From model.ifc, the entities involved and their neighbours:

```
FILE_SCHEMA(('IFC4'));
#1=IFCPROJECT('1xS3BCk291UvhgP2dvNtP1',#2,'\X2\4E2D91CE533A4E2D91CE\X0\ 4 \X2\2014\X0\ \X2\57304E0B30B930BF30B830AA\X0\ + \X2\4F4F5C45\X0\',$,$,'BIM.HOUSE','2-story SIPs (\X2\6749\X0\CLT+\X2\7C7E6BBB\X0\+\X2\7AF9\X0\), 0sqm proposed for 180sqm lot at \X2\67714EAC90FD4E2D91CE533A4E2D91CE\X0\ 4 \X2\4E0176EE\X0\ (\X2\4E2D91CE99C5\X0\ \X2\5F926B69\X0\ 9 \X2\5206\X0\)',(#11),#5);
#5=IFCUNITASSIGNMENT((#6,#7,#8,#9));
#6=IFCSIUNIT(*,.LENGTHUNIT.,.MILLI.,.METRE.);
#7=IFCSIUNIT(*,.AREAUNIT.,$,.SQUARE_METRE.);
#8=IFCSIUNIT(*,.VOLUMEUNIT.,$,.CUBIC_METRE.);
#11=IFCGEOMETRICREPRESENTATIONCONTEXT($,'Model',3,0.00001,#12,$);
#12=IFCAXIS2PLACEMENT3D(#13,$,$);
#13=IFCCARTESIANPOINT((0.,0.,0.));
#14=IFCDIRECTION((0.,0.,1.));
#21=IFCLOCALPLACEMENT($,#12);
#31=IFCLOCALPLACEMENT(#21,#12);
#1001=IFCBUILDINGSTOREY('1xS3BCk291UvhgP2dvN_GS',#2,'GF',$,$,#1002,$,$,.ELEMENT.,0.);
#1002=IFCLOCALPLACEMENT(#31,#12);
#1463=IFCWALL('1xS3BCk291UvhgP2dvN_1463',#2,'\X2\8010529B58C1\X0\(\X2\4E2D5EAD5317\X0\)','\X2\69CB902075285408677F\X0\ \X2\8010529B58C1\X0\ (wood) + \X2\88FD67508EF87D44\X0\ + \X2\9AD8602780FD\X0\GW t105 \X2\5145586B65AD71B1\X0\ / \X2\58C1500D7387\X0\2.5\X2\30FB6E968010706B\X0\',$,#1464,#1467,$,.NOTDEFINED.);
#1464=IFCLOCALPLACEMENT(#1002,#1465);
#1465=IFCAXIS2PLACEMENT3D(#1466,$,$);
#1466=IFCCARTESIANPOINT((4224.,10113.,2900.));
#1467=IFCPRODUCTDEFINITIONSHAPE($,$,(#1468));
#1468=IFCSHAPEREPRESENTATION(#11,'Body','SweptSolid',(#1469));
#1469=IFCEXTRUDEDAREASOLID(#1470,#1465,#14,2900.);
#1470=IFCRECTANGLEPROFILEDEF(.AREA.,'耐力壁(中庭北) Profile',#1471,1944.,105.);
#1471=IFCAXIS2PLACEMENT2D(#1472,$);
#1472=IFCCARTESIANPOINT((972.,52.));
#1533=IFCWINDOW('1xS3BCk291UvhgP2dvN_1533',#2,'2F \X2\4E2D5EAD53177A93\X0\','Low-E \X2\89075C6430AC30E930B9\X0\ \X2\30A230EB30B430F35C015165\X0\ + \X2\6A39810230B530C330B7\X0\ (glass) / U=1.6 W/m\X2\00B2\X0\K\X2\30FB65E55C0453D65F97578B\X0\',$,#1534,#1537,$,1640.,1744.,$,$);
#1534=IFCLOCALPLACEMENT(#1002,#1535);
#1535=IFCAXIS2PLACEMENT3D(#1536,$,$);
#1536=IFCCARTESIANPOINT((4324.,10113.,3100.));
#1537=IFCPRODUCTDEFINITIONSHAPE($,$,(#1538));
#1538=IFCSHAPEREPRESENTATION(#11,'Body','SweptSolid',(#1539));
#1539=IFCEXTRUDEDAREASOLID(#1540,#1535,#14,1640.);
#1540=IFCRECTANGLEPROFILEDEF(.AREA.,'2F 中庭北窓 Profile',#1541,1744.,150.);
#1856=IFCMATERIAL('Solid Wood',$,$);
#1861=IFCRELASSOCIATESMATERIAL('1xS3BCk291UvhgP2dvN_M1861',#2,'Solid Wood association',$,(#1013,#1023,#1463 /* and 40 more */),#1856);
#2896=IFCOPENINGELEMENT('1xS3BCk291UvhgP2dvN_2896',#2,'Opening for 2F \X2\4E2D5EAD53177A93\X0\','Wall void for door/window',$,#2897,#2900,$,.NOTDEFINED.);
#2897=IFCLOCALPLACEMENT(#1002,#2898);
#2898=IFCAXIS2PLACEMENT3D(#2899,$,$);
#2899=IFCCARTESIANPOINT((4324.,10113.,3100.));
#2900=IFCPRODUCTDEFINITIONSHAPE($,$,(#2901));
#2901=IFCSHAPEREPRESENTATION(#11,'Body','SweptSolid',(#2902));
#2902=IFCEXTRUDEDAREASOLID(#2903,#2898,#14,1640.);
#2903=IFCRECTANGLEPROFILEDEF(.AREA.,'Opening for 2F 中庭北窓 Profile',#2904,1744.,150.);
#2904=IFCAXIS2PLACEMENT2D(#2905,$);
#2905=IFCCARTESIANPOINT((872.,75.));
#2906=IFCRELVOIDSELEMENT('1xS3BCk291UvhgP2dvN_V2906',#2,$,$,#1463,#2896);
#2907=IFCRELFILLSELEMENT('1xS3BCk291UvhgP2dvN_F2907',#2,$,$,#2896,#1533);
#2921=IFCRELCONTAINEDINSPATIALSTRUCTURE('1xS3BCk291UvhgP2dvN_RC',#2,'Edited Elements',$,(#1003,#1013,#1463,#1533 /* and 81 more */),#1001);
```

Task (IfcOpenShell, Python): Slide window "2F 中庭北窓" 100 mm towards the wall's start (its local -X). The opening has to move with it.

```python
import ifcopenshell
import ifcopenshell.api.geometry
import ifcopenshell.util.placement

model = ifcopenshell.open("model.ifc")

window = model.by_id(1533)
opening = window.FillsVoids[0].RelatingOpeningElement
wall = opening.VoidsElements[0].RelatingBuildingElement

wall_matrix = ifcopenshell.util.placement.get_local_placement(wall.ObjectPlacement)
shift = wall_matrix[:3, 0] * -100.0
before = ifcopenshell.util.placement.get_local_placement(window.ObjectPlacement)[:3, 3].copy()

# The window is not placed relative to its opening, so move both.
for product in (opening, window):
    matrix = ifcopenshell.util.placement.get_local_placement(product.ObjectPlacement)
    matrix[:3, 3] += shift
    ifcopenshell.api.geometry.edit_object_placement(model, product=product, matrix=matrix, is_si=False)

after = ifcopenshell.util.placement.get_local_placement(window.ObjectPlacement)[:3, 3]
print("window moved by", (after - before).round(3) + 0.0)

model.write("model_rev.ifc")
```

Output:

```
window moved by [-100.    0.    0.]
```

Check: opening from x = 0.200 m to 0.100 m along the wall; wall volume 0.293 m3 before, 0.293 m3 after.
